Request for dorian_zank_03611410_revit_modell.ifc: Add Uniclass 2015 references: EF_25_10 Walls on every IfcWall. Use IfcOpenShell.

First a look at what the model holds.

```python
import ifcopenshell

model = ifcopenshell.open("dorian_zank_03611410_revit_modell.ifc")
print(model.schema)
print("classifications:", [c.Name for c in model.by_type("IfcClassification")])
for ifc_class in ("IfcDoor", "IfcRoof", "IfcStair", "IfcWall", "IfcWindow"):
    print(ifc_class, len(model.by_type(ifc_class)))
```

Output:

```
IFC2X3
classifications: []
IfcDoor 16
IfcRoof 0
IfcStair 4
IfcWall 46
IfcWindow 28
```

```python
import ifcopenshell
import ifcopenshell.api.classification

model = ifcopenshell.open("dorian_zank_03611410_revit_modell.ifc")

# IFC2X3 requires Source and Edition and has no link from the project to the system.
system = model.create_entity("IfcClassification", Source="NBS", Edition="2015", Name="Uniclass 2015")

codes = {
    "IfcWall": ("EF_25_10", "Walls"),
}
for ifc_class, (code, name) in codes.items():
    products = model.by_type(ifc_class)
    ifcopenshell.api.classification.add_reference(
        model, products=products, classification=system, identification=code, name=name
    )
    print(code, len(products))

model.write("dorian_zank_03611410_revit_modell_v2.ifc")
```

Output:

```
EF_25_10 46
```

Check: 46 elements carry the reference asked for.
